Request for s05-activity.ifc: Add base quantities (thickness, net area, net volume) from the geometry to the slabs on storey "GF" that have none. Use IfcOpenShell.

First a look at what the model holds.

```python
import ifcopenshell
import ifcopenshell.util.element
import ifcopenshell.util.unit

model = ifcopenshell.open("s05-activity.ifc")
print(model.schema)
for unit_type in ("LENGTHUNIT", "AREAUNIT", "VOLUMEUNIT"):
    print(unit_type, ifcopenshell.util.unit.calculate_unit_scale(model, unit_type))
storey = next(s for s in model.by_type("IfcBuildingStorey") if s.Name == "GF")
slabs = [e for e in ifcopenshell.util.element.get_decomposition(storey) if e.is_a("IfcSlab")]
for e in sorted(slabs, key=lambda e: e.id()):
    print(e.id(), e.is_a(), e.Name, list(ifcopenshell.util.element.get_psets(e, qtos_only=True)), sep=" | ")
```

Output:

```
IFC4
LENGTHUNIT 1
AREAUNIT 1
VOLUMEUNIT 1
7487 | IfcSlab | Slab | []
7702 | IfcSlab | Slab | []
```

```python
import ifcopenshell
import ifcopenshell.api.pset
import ifcopenshell.geom
import ifcopenshell.util.element
import ifcopenshell.util.shape
import ifcopenshell.util.unit

model = ifcopenshell.open("s05-activity.ifc")
unit_scale = ifcopenshell.util.unit.calculate_unit_scale(model)
area_scale = ifcopenshell.util.unit.calculate_unit_scale(model, "AREAUNIT")
volume_scale = ifcopenshell.util.unit.calculate_unit_scale(model, "VOLUMEUNIT")
settings = ifcopenshell.geom.settings()

storey = next(s for s in model.by_type("IfcBuildingStorey") if s.Name == "GF")
slabs = [e for e in ifcopenshell.util.element.get_decomposition(storey) if e.is_a("IfcSlab")]

for e in sorted(slabs, key=lambda e: e.id()):
    if ifcopenshell.util.element.get_psets(e, qtos_only=True, should_inherit=False):
        continue
    # Geometry comes back in metres, in the element's own axes.
    shape = ifcopenshell.geom.create_shape(settings, e)
    values = {
        "Width": ifcopenshell.util.shape.get_z(shape.geometry) / unit_scale,
        "NetArea": ifcopenshell.util.shape.get_footprint_area(shape.geometry) / area_scale,
        "NetVolume": ifcopenshell.util.shape.get_volume(shape.geometry) / volume_scale,
    }
    qto = ifcopenshell.api.pset.add_qto(model, product=e, name="Qto_SlabBaseQuantities")
    ifcopenshell.api.pset.edit_qto(model, qto=qto, properties=values)
    print(e.id(), {k: round(v, 3) for k, v in values.items()})

model.write("s05-activity_v2.ifc")
```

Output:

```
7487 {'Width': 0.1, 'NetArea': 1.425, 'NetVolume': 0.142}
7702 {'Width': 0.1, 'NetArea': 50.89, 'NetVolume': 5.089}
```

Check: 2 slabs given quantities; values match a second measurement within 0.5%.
